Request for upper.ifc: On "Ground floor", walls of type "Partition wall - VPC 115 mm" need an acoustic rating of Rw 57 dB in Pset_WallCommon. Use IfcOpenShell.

First a look at what the model holds.

```python
import ifcopenshell
import ifcopenshell.util.element

model = ifcopenshell.open("upper.ifc")
print(model.schema)
storey = next(s for s in model.by_type("IfcBuildingStorey") if s.Name == "Ground floor")
walls = [e for e in ifcopenshell.util.element.get_decomposition(storey) if e.is_a("IfcWall")]
seen = {}
for e in walls:
    element_type = ifcopenshell.util.element.get_type(e)
    key = (element_type.Name if element_type != e and element_type else None, ifcopenshell.util.element.get_pset(e, "Pset_WallCommon", "AcousticRating"))
    seen[key] = seen.get(key, 0) + 1
for (name, value), count in sorted(seen.items(), key=str):
    print(count, "x", name, "|", value)
```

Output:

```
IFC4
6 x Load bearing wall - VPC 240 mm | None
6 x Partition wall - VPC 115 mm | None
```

```python
import ifcopenshell
import ifcopenshell.api.pset
import ifcopenshell.util.element

model = ifcopenshell.open("upper.ifc")

storey = next(s for s in model.by_type("IfcBuildingStorey") if s.Name == "Ground floor")
walls = [e for e in ifcopenshell.util.element.get_decomposition(storey) if e.is_a("IfcWall")]

count = 0
for e in walls:
    element_type = ifcopenshell.util.element.get_type(e)
    if element_type in (None, e) or element_type.Name != "Partition wall - VPC 115 mm":
        continue
    # add_pset returns the element's existing set when there is one.
    pset = ifcopenshell.api.pset.add_pset(model, product=e, name="Pset_WallCommon")
    ifcopenshell.api.pset.edit_pset(model, pset=pset, properties={"AcousticRating": "Rw 57 dB"})
    count += 1

print(count, "walls updated")

model.write("upper_rev.ifc")
```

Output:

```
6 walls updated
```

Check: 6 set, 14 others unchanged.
